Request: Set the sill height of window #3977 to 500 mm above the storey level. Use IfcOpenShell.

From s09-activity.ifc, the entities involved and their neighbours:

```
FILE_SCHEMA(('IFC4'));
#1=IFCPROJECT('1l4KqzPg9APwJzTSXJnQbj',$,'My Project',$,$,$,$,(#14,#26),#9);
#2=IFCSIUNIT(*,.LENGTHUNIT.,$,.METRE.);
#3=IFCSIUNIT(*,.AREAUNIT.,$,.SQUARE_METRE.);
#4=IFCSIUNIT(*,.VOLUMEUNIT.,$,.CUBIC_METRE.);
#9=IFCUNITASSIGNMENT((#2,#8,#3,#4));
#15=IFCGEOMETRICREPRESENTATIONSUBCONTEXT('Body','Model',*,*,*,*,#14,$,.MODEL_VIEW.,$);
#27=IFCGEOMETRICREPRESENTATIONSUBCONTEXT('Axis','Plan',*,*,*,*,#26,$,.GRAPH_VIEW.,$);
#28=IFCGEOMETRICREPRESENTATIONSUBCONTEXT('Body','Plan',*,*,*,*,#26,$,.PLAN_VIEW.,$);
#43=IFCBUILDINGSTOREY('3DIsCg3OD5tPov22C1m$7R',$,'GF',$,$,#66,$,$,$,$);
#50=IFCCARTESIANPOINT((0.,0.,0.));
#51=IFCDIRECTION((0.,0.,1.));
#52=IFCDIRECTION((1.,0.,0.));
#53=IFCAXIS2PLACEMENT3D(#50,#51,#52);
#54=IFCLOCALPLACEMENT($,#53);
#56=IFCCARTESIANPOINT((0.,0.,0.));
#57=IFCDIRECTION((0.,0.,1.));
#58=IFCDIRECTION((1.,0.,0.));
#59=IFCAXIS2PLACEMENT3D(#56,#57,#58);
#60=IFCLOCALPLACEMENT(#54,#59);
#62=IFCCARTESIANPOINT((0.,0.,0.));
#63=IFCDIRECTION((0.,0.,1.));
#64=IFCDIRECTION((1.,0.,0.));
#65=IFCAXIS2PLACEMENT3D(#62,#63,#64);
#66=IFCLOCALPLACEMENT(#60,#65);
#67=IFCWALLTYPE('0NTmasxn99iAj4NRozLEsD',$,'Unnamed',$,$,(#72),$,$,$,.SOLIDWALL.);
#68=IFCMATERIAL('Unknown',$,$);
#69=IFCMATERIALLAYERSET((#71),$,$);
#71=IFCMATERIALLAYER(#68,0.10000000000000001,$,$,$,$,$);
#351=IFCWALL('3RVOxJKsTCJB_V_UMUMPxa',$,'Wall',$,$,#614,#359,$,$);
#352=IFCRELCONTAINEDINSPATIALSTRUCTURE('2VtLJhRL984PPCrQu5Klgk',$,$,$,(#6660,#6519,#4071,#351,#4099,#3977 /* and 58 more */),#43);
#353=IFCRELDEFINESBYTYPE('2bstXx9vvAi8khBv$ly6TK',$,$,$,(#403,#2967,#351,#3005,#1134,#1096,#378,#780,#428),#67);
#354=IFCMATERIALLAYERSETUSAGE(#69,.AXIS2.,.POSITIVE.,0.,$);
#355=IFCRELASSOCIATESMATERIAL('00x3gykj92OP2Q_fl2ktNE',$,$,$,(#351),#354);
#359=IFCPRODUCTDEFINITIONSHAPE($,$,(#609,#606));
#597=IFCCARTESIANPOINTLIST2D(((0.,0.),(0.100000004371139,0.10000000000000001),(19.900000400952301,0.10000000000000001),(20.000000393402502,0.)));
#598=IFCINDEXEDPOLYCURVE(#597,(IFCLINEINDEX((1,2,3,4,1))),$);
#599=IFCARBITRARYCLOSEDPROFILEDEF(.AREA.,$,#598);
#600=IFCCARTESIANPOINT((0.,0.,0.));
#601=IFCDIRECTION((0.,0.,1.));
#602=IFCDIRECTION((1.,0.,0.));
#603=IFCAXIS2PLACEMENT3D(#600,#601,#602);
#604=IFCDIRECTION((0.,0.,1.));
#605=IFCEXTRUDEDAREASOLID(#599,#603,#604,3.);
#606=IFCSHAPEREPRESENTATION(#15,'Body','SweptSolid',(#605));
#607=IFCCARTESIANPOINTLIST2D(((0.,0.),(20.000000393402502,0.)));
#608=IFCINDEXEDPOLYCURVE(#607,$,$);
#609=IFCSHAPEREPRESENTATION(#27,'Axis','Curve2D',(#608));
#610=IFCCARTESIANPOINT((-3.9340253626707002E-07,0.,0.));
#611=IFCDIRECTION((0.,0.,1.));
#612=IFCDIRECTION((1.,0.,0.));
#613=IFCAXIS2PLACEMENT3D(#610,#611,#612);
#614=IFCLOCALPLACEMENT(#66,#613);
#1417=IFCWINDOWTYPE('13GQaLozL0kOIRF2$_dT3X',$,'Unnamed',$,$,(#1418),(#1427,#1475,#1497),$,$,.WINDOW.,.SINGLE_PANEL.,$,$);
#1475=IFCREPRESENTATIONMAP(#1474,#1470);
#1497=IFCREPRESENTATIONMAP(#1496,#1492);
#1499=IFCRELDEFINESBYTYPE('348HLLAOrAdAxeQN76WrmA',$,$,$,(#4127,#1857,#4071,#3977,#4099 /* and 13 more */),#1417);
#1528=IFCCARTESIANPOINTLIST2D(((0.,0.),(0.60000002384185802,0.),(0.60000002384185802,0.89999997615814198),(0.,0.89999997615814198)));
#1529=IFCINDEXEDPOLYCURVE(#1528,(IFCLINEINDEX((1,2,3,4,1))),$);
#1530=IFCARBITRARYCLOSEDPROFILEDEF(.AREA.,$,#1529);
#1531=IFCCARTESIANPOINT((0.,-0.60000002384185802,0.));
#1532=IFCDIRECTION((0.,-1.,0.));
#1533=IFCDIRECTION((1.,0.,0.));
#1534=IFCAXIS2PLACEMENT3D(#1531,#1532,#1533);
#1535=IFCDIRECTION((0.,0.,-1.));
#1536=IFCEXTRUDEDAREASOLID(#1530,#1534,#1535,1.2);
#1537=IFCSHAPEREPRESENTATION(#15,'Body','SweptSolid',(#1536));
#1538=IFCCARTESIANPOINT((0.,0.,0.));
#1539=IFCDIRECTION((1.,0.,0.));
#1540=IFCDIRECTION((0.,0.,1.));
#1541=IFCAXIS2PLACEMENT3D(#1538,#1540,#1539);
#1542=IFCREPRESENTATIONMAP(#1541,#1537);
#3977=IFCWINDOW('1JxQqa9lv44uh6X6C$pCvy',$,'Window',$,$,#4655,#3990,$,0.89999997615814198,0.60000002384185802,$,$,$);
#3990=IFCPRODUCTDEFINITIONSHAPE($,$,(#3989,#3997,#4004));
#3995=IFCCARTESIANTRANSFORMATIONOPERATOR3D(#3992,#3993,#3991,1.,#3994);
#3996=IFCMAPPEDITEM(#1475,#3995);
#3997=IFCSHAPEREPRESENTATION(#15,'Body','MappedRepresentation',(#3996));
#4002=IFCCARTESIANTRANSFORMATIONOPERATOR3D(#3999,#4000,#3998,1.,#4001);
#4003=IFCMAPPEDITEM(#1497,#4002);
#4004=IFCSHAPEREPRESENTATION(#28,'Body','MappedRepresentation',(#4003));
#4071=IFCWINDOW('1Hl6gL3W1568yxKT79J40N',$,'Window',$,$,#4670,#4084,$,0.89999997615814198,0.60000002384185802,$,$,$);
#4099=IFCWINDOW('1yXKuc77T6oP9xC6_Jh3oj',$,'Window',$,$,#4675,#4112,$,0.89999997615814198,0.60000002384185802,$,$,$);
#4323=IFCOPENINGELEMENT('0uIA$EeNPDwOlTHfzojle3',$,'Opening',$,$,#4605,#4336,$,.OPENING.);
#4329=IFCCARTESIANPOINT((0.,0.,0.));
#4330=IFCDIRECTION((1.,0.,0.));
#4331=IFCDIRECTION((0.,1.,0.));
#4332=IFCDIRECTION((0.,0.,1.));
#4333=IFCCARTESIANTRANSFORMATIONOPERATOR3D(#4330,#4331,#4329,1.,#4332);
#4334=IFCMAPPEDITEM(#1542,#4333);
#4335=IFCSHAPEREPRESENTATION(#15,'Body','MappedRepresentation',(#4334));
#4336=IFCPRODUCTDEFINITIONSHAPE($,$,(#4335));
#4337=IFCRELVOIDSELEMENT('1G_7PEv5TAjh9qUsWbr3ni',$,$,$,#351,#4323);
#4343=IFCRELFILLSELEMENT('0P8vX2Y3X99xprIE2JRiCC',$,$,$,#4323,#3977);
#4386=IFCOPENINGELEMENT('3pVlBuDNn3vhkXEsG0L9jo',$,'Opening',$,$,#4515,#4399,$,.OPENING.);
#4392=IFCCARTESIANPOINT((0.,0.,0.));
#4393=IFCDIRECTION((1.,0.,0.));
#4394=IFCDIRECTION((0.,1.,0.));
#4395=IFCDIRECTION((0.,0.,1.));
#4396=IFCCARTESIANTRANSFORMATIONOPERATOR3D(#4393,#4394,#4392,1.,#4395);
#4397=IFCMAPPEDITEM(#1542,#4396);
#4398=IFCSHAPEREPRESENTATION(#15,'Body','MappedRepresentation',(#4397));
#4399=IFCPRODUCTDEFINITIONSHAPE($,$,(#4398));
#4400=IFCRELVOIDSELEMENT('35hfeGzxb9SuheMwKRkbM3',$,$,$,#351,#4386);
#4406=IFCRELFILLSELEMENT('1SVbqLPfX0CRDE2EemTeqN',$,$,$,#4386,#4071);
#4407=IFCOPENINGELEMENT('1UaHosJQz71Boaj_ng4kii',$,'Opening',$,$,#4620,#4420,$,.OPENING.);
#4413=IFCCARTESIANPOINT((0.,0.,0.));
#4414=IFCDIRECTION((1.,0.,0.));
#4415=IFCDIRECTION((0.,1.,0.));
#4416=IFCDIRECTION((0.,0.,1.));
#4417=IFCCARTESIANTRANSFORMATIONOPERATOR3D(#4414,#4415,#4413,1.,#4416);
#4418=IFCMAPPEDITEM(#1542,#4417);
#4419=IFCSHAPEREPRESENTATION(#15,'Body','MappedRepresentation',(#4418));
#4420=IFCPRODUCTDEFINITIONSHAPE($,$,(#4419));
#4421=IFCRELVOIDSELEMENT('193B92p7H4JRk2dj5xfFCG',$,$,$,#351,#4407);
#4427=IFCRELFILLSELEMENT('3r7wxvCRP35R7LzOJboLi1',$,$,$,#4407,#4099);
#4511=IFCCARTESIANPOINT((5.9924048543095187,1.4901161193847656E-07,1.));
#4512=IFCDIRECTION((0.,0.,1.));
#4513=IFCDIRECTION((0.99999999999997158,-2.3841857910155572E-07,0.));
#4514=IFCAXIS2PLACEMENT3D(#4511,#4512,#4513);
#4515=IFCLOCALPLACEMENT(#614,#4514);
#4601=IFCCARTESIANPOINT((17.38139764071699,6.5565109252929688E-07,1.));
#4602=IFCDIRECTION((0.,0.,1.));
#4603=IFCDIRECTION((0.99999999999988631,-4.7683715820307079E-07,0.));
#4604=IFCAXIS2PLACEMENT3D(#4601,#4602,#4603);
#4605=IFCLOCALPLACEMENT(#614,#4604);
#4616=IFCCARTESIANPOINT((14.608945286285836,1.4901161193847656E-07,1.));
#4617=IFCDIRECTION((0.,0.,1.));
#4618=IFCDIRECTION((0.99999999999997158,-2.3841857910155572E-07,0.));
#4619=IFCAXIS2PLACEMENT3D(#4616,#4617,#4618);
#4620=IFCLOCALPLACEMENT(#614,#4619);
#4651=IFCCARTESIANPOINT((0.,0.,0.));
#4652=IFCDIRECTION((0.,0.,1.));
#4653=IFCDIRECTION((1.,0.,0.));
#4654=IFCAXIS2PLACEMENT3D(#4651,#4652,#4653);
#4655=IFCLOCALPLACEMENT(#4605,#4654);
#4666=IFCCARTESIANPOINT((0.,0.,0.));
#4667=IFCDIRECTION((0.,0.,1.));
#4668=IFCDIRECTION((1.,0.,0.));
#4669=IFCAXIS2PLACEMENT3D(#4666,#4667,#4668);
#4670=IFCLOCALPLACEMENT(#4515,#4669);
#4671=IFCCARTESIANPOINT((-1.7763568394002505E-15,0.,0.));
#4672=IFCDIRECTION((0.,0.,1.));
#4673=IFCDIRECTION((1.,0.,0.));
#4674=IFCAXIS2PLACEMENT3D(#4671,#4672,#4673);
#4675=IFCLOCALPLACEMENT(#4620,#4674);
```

```python
import numpy as np
import ifcopenshell
import ifcopenshell.api.geometry
import ifcopenshell.geom
import ifcopenshell.util.element
import ifcopenshell.util.placement
import ifcopenshell.util.shape
import ifcopenshell.util.unit

model = ifcopenshell.open("s09-activity.ifc")
unit_scale = ifcopenshell.util.unit.calculate_unit_scale(model)

window = model.by_guid("1JxQqa9lv44uh6X6C$pCvy")
opening = window.FillsVoids[0].RelatingOpeningElement
storey = ifcopenshell.util.element.get_container(window, ifc_class="IfcBuildingStorey")
level = ifcopenshell.util.placement.get_local_placement(storey.ObjectPlacement)[2, 3]

# The opening's origin need not be at the sill, so measure its lowest point.
shape = ifcopenshell.geom.create_shape(ifcopenshell.geom.settings(), opening)
bottom = ifcopenshell.util.shape.get_shape_bottom_elevation(shape, shape.geometry) / unit_scale
dz = level + 0.5 / unit_scale - bottom

shift = np.array([0.0, 0.0, dz])
# The window is placed relative to its opening, so it follows when the opening moves.
matrix = ifcopenshell.util.placement.get_local_placement(opening.ObjectPlacement)
matrix[:3, 3] += shift
ifcopenshell.api.geometry.edit_object_placement(
    model, product=opening, matrix=matrix, is_si=False, should_transform_children=True
)

print(f"moved by {dz * unit_scale:+.3f} m")

model.write("s09-activity_rev.ifc")
```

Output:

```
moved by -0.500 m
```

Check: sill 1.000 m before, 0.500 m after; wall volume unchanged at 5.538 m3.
